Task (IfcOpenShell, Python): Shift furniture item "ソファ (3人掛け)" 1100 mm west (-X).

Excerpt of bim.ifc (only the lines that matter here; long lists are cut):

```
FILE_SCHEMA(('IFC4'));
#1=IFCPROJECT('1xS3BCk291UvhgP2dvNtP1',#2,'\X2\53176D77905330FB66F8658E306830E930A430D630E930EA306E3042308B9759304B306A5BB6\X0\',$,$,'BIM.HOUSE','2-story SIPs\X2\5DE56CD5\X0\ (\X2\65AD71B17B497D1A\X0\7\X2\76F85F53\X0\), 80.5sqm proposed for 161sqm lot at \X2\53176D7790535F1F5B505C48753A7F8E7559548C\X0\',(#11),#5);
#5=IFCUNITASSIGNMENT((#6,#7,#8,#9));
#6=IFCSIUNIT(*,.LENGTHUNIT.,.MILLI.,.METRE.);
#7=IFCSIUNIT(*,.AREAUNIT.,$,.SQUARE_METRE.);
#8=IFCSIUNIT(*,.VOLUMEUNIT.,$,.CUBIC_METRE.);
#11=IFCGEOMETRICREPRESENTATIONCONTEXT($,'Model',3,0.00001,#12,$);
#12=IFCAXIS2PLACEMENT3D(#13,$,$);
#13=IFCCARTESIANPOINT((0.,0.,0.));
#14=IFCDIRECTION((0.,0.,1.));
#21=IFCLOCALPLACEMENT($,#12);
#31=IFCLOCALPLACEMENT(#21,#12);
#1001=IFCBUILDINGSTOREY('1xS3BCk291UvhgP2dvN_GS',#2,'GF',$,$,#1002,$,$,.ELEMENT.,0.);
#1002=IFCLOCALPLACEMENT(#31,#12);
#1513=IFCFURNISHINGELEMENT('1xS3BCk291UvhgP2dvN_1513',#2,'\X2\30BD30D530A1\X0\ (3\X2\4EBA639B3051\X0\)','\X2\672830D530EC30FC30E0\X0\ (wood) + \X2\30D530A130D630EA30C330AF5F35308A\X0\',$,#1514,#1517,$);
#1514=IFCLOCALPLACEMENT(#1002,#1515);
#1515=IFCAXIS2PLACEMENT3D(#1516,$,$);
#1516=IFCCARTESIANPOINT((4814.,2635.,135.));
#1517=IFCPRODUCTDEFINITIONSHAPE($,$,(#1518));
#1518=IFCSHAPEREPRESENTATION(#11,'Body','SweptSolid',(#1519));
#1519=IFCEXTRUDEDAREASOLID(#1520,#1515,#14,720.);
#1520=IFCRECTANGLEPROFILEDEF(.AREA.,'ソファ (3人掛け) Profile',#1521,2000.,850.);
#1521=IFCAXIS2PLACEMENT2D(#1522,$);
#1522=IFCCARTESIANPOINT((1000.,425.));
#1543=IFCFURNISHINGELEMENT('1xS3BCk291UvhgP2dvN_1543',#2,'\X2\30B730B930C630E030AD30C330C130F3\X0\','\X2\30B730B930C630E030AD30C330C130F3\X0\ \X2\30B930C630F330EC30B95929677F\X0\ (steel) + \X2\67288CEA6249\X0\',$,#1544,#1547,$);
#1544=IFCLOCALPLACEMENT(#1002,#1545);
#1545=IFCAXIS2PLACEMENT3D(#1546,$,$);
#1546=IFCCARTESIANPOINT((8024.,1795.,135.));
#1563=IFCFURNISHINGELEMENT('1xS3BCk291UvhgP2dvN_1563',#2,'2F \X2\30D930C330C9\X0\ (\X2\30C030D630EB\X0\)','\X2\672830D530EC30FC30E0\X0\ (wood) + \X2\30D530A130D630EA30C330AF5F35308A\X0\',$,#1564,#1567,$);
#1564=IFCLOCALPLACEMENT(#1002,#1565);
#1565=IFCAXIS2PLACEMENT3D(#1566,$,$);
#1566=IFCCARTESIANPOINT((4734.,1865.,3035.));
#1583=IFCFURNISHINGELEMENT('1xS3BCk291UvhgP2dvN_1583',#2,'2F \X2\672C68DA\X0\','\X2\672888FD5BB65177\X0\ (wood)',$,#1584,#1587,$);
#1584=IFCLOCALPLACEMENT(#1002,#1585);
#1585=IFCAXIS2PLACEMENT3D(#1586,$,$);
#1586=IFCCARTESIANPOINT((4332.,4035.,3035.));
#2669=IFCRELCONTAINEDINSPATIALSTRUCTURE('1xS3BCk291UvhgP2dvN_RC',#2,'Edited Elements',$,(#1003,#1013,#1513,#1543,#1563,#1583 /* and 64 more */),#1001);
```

```python
import ifcopenshell
import ifcopenshell.api.geometry
import ifcopenshell.util.placement

model = ifcopenshell.open("bim.ifc")

item = model.by_id(1513)
matrix = ifcopenshell.util.placement.get_local_placement(item.ObjectPlacement)
matrix[0, 3] -= 1100.0
ifcopenshell.api.geometry.edit_object_placement(model, product=item, matrix=matrix, is_si=False)

print(ifcopenshell.util.placement.get_local_placement(item.ObjectPlacement).round(3) + 0.0)

model.write("bim_edited.ifc")
```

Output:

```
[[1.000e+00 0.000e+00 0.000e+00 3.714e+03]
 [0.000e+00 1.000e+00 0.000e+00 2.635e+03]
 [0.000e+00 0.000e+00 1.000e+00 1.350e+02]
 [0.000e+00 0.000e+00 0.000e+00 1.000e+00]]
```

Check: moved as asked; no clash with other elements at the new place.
